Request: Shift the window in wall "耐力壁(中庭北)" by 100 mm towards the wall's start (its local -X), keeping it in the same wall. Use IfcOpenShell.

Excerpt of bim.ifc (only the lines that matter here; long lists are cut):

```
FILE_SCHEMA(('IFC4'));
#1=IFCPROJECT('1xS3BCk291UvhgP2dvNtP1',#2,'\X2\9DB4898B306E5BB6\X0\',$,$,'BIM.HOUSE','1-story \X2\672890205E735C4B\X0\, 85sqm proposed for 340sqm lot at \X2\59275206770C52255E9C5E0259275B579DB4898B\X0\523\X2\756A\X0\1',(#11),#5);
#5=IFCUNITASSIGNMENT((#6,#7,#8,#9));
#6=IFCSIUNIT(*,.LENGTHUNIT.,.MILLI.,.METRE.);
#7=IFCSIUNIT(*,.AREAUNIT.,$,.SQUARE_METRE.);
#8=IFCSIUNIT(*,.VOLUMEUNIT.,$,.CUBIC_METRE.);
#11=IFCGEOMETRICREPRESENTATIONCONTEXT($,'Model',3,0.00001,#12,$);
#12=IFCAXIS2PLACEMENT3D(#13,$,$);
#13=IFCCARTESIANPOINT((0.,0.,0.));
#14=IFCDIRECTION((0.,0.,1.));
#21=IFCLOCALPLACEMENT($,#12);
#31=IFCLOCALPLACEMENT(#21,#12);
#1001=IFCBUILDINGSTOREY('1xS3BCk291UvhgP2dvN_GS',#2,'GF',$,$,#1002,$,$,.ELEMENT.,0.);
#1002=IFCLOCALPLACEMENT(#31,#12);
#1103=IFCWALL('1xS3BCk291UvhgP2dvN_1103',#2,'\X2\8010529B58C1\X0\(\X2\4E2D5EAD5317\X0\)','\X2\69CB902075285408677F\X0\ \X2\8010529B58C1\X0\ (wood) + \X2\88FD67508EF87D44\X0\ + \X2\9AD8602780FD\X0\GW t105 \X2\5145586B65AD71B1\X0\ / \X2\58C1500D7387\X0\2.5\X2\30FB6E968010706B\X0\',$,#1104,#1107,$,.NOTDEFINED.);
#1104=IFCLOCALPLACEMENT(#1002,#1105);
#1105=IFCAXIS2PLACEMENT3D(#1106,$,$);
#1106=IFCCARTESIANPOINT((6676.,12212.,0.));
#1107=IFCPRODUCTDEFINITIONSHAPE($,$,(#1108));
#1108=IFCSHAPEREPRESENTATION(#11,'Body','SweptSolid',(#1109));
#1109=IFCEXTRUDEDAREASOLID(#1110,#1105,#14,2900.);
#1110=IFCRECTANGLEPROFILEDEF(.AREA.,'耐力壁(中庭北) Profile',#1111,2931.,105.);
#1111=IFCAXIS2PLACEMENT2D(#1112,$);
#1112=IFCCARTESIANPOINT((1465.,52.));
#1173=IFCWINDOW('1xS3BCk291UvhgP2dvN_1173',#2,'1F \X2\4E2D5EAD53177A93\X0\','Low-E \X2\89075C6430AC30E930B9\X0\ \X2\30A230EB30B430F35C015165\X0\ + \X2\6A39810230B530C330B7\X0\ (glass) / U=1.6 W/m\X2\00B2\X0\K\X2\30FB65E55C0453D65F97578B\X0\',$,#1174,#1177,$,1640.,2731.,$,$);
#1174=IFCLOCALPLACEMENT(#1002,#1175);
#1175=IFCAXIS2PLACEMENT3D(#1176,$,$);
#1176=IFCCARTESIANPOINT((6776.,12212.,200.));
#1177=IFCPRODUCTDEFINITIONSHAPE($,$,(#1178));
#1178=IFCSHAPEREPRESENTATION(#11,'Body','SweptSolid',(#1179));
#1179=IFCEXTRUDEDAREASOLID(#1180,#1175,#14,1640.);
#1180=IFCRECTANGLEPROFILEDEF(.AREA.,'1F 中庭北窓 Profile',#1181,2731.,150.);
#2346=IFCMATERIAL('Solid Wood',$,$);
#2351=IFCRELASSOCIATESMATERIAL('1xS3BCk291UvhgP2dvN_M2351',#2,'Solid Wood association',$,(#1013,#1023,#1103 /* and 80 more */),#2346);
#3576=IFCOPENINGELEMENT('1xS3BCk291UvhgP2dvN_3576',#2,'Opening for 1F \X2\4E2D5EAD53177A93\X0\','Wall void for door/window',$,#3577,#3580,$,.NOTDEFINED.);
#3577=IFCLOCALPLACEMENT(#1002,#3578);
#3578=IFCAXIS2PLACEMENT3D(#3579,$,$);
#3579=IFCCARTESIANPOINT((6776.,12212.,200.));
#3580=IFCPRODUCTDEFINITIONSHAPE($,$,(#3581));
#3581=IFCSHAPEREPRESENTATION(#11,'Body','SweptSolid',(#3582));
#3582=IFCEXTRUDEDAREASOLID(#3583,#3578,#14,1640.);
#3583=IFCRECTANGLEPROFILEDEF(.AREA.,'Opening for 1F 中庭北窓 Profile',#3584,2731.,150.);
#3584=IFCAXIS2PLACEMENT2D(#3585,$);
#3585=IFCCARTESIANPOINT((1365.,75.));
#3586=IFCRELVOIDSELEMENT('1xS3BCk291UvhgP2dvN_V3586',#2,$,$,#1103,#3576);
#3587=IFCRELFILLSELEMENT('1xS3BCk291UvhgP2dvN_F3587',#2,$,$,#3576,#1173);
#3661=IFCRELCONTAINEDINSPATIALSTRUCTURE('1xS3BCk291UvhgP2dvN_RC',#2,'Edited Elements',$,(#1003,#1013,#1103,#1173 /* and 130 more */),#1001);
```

```python
import ifcopenshell
import ifcopenshell.api.geometry
import ifcopenshell.util.placement
import ifcopenshell.util.unit

model = ifcopenshell.open("bim.ifc")
unit_scale = ifcopenshell.util.unit.calculate_unit_scale(model)

window = model.by_id(1173)
opening = window.FillsVoids[0].RelatingOpeningElement
wall = opening.VoidsElements[0].RelatingBuildingElement

wall_matrix = ifcopenshell.util.placement.get_local_placement(wall.ObjectPlacement)
shift = wall_matrix[:3, 0] * -0.1 / unit_scale
before = ifcopenshell.util.placement.get_local_placement(window.ObjectPlacement)[:3, 3].copy()

# The window is not placed relative to its opening, so move both.
for product in (opening, window):
    matrix = ifcopenshell.util.placement.get_local_placement(product.ObjectPlacement)
    matrix[:3, 3] += shift
    ifcopenshell.api.geometry.edit_object_placement(model, product=product, matrix=matrix, is_si=False)

after = ifcopenshell.util.placement.get_local_placement(window.ObjectPlacement)[:3, 3]
print("window moved by", (after - before).round(3) + 0.0)

model.write("bim_edited.ifc")
```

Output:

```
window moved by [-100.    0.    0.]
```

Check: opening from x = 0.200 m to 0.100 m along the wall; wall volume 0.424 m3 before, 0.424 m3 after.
